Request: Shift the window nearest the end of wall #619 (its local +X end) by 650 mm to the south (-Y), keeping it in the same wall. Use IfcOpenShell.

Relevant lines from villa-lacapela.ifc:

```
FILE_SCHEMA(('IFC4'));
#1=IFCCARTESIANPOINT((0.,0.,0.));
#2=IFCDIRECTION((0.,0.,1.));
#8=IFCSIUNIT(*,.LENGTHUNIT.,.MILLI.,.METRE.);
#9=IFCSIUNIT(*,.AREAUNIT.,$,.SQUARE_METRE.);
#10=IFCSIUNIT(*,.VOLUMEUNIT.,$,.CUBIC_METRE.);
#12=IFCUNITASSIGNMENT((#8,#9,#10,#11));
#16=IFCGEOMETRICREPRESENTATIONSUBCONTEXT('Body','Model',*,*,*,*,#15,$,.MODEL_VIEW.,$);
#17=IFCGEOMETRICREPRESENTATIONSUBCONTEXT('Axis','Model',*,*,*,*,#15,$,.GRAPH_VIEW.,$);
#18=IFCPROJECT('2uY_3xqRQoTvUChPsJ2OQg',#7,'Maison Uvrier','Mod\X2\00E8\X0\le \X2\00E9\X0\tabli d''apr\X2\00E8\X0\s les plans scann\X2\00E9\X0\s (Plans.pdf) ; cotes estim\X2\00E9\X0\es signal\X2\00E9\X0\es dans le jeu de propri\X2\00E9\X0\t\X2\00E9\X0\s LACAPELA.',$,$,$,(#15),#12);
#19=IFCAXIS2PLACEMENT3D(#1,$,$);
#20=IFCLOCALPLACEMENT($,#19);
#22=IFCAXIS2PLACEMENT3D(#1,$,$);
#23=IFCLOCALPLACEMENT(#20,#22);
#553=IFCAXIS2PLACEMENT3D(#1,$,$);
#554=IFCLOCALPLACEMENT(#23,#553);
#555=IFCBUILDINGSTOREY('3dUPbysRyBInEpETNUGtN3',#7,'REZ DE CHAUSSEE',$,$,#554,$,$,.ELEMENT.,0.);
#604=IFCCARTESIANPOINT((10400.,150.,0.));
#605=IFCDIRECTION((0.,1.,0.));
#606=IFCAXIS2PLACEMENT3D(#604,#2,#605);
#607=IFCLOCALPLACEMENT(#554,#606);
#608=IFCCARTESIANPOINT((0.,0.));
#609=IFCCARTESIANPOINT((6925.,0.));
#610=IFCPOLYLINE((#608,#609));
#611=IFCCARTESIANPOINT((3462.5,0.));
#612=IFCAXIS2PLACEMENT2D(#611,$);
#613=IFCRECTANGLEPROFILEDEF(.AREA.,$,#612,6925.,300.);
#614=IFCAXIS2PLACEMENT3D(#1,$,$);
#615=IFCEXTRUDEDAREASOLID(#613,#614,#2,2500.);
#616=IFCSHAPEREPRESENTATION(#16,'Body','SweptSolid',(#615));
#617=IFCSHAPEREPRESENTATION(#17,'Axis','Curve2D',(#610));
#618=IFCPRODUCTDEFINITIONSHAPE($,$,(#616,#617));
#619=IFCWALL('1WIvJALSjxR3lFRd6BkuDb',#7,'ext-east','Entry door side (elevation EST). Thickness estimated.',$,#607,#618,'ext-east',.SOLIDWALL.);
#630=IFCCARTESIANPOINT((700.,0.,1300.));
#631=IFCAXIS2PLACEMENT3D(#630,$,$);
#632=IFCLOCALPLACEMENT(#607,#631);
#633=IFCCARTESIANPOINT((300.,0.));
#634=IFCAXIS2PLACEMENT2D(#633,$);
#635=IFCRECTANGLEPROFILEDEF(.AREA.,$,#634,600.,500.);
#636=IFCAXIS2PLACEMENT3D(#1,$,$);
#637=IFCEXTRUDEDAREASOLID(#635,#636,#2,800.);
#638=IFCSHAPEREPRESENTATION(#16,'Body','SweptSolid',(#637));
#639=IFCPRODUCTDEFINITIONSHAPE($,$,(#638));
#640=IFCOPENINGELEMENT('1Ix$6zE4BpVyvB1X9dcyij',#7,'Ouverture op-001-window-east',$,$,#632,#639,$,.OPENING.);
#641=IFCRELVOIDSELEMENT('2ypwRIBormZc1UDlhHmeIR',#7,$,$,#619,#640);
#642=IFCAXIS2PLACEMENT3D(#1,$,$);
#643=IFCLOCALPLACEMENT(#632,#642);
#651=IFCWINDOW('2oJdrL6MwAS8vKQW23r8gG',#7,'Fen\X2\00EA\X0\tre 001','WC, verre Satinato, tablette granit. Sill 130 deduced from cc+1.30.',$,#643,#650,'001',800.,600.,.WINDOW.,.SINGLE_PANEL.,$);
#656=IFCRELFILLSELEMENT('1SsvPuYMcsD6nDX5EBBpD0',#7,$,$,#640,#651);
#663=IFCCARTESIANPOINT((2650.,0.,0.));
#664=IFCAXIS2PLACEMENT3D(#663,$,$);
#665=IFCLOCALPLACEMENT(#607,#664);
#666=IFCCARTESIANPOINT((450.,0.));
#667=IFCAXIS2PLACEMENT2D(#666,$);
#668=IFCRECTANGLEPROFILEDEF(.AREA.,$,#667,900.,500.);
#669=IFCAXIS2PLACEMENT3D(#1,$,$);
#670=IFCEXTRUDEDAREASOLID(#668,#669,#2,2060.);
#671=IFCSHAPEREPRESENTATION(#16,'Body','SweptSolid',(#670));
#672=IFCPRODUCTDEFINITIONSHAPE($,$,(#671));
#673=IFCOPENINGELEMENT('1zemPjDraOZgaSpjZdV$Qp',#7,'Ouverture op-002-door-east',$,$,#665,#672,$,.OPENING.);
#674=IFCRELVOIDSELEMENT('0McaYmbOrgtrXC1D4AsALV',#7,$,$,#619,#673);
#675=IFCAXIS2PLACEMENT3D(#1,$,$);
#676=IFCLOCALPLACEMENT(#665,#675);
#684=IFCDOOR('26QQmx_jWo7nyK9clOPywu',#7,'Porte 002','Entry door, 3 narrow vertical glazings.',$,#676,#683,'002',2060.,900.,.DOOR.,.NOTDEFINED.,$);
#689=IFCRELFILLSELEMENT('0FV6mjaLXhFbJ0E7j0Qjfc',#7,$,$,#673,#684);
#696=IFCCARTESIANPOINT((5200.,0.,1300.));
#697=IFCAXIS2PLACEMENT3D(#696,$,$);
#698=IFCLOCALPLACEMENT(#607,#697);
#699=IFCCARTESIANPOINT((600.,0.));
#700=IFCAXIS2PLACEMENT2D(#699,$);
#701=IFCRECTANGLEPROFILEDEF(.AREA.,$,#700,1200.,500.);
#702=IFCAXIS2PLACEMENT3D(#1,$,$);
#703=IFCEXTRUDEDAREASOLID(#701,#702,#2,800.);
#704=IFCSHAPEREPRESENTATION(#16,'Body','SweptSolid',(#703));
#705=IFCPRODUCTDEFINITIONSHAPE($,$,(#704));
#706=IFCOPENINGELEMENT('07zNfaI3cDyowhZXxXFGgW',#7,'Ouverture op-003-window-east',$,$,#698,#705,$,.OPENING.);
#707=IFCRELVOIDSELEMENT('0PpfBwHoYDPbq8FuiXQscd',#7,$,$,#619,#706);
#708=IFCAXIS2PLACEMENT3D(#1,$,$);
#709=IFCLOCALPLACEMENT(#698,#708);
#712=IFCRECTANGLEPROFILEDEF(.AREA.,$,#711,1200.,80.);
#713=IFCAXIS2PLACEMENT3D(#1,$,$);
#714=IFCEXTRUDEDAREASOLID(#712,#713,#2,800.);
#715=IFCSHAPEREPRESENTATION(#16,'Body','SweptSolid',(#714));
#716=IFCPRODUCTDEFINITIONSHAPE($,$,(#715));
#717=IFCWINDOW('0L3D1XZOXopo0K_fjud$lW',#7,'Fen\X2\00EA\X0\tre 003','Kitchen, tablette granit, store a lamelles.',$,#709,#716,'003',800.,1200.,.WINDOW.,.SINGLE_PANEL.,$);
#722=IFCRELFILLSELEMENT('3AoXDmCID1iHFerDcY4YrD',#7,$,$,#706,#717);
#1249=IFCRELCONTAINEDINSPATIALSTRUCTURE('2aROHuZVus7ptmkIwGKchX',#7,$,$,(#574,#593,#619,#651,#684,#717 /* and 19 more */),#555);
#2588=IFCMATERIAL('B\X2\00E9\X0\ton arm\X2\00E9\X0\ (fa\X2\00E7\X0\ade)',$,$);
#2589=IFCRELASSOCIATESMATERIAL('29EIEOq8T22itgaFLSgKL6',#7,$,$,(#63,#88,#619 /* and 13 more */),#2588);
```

```python
import ifcopenshell
import ifcopenshell.api.geometry
import ifcopenshell.util.placement

model = ifcopenshell.open("villa-lacapela.ifc")

window = model.by_id(717)
opening = window.FillsVoids[0].RelatingOpeningElement
wall = opening.VoidsElements[0].RelatingBuildingElement

wall_matrix = ifcopenshell.util.placement.get_local_placement(wall.ObjectPlacement)
shift = wall_matrix[:3, 0] * -650.0
before = ifcopenshell.util.placement.get_local_placement(window.ObjectPlacement)[:3, 3].copy()

# The window is placed relative to its opening, so it follows when the opening moves.
matrix = ifcopenshell.util.placement.get_local_placement(opening.ObjectPlacement)
matrix[:3, 3] += shift
ifcopenshell.api.geometry.edit_object_placement(
    model, product=opening, matrix=matrix, is_si=False, should_transform_children=True
)

after = ifcopenshell.util.placement.get_local_placement(window.ObjectPlacement)[:3, 3]
print("window moved by", (after - before).round(3) + 0.0)

model.write("villa-lacapela-out.ifc")
```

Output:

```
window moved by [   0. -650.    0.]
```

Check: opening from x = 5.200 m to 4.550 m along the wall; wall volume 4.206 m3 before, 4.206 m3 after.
